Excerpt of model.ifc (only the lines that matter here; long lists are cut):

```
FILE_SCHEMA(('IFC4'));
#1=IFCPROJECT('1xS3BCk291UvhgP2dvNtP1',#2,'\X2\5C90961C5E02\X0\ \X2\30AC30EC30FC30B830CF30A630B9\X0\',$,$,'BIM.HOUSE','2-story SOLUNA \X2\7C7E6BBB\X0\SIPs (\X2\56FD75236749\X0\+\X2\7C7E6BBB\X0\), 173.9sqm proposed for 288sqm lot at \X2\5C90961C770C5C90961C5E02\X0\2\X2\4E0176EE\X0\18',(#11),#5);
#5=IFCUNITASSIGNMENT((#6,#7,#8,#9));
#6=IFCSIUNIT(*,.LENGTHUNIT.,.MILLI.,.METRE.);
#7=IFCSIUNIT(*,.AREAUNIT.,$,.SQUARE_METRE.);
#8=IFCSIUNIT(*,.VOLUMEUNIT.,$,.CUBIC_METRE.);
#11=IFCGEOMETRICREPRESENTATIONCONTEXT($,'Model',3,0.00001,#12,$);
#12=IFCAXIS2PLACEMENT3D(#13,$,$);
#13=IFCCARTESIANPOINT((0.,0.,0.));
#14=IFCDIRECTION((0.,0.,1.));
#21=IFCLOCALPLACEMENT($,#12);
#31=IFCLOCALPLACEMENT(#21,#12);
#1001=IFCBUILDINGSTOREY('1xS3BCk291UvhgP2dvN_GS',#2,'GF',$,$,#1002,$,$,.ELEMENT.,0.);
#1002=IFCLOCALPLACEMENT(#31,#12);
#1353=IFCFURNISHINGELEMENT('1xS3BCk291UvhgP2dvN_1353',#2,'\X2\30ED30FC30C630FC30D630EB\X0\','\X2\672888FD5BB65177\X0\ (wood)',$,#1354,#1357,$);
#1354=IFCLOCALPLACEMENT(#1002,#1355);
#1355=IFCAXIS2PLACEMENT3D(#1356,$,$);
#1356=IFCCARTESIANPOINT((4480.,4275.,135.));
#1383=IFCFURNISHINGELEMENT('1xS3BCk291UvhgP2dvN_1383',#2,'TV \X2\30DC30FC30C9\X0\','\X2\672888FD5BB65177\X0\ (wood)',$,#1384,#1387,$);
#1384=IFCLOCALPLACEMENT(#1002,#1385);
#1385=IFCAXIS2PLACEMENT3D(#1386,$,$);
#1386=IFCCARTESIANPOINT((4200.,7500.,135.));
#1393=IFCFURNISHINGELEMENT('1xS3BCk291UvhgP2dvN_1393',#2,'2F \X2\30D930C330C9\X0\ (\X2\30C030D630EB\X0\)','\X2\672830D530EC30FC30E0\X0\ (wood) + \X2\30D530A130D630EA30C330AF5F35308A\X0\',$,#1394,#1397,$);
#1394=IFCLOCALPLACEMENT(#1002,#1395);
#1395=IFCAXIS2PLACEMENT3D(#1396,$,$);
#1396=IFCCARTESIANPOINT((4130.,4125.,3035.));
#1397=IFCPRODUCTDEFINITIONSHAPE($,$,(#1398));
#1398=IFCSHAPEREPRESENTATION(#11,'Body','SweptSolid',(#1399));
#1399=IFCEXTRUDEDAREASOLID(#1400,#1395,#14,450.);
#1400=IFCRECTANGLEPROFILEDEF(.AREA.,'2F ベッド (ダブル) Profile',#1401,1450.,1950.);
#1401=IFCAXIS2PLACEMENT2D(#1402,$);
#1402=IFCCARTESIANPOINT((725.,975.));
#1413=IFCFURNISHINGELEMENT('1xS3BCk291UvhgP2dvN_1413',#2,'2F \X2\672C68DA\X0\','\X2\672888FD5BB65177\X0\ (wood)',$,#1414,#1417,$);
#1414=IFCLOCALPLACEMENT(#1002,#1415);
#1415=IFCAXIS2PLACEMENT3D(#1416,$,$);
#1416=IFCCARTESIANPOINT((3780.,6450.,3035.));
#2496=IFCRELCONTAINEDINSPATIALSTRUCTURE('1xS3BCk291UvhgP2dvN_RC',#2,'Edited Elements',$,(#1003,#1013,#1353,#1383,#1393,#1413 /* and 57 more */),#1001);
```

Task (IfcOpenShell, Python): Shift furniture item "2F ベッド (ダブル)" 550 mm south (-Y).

```python
import ifcopenshell
import ifcopenshell.api.geometry
import ifcopenshell.util.placement

model = ifcopenshell.open("model.ifc")

item = model.by_id(1393)
matrix = ifcopenshell.util.placement.get_local_placement(item.ObjectPlacement)
matrix[1, 3] -= 550.0
ifcopenshell.api.geometry.edit_object_placement(model, product=item, matrix=matrix, is_si=False)

print(ifcopenshell.util.placement.get_local_placement(item.ObjectPlacement).round(3) + 0.0)

model.write("model_rev.ifc")
```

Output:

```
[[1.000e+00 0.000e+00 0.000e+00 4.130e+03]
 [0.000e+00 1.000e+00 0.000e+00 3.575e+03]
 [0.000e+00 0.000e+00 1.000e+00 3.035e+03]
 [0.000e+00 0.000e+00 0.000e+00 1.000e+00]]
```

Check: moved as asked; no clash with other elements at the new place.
